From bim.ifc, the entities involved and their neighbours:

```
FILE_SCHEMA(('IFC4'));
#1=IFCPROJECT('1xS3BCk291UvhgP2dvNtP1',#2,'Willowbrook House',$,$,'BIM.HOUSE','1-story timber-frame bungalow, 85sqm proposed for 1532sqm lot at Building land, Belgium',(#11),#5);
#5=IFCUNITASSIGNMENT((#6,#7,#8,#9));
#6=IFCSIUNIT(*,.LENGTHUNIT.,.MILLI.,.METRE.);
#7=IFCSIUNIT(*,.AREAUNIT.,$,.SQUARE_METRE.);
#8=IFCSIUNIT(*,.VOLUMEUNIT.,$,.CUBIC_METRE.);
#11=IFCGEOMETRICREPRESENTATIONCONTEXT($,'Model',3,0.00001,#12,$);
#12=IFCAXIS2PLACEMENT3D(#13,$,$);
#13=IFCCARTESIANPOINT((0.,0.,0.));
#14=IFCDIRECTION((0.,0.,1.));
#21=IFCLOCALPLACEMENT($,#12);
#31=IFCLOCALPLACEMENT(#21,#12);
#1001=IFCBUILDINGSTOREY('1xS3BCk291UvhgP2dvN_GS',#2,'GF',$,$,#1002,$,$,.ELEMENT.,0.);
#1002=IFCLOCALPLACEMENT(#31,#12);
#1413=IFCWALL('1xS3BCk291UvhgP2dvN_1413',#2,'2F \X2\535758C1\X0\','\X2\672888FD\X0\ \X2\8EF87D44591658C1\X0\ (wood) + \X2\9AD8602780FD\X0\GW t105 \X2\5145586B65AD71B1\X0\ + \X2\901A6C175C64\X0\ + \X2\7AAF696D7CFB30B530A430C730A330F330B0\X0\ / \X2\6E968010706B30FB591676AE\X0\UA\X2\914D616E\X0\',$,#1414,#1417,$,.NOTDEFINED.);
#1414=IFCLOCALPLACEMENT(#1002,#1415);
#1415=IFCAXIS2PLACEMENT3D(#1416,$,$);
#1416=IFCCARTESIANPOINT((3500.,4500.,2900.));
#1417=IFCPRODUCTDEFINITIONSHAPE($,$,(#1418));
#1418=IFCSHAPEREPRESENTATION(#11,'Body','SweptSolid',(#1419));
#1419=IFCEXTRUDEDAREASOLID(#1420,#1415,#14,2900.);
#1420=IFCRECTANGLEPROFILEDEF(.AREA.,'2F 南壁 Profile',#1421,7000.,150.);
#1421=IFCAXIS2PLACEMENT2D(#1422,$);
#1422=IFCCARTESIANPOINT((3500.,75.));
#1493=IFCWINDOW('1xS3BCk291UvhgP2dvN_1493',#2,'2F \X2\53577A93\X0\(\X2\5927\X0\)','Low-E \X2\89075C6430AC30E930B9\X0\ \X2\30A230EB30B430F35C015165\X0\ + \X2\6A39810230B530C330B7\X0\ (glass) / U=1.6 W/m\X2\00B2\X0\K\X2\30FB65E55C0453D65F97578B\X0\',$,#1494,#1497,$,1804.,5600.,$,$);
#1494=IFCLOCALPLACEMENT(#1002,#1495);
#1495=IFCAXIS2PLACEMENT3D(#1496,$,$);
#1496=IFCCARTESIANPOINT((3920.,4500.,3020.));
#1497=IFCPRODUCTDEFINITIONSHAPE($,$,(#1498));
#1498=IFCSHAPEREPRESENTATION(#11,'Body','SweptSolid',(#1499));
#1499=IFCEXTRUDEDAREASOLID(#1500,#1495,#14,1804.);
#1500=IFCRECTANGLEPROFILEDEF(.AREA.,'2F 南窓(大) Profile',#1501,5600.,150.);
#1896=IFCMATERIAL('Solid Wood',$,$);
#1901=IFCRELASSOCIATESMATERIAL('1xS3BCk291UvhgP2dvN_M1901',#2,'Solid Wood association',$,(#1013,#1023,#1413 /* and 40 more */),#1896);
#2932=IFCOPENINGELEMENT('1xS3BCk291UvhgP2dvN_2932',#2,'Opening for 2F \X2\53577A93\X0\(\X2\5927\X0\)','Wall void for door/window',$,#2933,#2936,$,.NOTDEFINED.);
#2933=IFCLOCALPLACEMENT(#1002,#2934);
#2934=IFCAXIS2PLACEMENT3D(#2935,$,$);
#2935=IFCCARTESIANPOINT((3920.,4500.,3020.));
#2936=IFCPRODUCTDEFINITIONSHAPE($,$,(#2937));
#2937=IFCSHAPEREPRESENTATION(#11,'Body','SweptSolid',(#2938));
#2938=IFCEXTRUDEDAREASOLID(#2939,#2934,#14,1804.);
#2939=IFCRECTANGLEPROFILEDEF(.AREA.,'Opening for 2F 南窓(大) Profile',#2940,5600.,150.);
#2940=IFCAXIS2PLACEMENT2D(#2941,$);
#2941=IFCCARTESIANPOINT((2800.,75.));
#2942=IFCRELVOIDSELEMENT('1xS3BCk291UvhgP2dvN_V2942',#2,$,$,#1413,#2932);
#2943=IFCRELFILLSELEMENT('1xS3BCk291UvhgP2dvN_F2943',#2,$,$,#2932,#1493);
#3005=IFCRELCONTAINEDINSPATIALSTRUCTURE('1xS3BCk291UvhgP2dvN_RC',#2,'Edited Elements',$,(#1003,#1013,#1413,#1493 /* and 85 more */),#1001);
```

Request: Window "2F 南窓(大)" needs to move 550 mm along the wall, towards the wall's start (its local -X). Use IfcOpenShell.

```python
import ifcopenshell
import ifcopenshell.api.geometry
import ifcopenshell.util.placement
import ifcopenshell.util.unit

model = ifcopenshell.open("bim.ifc")
unit_scale = ifcopenshell.util.unit.calculate_unit_scale(model)

window = model.by_guid("1xS3BCk291UvhgP2dvN_1493")
opening = window.FillsVoids[0].RelatingOpeningElement
wall = opening.VoidsElements[0].RelatingBuildingElement

wall_matrix = ifcopenshell.util.placement.get_local_placement(wall.ObjectPlacement)
shift = wall_matrix[:3, 0] * -0.55 / unit_scale
before = ifcopenshell.util.placement.get_local_placement(window.ObjectPlacement)[:3, 3].copy()

# The window is not placed relative to its opening, so move both.
for product in (opening, window):
    matrix = ifcopenshell.util.placement.get_local_placement(product.ObjectPlacement)
    matrix[:3, 3] += shift
    ifcopenshell.api.geometry.edit_object_placement(model, product=product, matrix=matrix, is_si=False)

after = ifcopenshell.util.placement.get_local_placement(window.ObjectPlacement)[:3, 3]
print("window moved by", (after - before).round(3) + 0.0)

model.write("bim_updated.ifc")
```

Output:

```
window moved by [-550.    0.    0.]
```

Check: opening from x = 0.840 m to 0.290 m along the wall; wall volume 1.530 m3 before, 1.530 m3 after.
